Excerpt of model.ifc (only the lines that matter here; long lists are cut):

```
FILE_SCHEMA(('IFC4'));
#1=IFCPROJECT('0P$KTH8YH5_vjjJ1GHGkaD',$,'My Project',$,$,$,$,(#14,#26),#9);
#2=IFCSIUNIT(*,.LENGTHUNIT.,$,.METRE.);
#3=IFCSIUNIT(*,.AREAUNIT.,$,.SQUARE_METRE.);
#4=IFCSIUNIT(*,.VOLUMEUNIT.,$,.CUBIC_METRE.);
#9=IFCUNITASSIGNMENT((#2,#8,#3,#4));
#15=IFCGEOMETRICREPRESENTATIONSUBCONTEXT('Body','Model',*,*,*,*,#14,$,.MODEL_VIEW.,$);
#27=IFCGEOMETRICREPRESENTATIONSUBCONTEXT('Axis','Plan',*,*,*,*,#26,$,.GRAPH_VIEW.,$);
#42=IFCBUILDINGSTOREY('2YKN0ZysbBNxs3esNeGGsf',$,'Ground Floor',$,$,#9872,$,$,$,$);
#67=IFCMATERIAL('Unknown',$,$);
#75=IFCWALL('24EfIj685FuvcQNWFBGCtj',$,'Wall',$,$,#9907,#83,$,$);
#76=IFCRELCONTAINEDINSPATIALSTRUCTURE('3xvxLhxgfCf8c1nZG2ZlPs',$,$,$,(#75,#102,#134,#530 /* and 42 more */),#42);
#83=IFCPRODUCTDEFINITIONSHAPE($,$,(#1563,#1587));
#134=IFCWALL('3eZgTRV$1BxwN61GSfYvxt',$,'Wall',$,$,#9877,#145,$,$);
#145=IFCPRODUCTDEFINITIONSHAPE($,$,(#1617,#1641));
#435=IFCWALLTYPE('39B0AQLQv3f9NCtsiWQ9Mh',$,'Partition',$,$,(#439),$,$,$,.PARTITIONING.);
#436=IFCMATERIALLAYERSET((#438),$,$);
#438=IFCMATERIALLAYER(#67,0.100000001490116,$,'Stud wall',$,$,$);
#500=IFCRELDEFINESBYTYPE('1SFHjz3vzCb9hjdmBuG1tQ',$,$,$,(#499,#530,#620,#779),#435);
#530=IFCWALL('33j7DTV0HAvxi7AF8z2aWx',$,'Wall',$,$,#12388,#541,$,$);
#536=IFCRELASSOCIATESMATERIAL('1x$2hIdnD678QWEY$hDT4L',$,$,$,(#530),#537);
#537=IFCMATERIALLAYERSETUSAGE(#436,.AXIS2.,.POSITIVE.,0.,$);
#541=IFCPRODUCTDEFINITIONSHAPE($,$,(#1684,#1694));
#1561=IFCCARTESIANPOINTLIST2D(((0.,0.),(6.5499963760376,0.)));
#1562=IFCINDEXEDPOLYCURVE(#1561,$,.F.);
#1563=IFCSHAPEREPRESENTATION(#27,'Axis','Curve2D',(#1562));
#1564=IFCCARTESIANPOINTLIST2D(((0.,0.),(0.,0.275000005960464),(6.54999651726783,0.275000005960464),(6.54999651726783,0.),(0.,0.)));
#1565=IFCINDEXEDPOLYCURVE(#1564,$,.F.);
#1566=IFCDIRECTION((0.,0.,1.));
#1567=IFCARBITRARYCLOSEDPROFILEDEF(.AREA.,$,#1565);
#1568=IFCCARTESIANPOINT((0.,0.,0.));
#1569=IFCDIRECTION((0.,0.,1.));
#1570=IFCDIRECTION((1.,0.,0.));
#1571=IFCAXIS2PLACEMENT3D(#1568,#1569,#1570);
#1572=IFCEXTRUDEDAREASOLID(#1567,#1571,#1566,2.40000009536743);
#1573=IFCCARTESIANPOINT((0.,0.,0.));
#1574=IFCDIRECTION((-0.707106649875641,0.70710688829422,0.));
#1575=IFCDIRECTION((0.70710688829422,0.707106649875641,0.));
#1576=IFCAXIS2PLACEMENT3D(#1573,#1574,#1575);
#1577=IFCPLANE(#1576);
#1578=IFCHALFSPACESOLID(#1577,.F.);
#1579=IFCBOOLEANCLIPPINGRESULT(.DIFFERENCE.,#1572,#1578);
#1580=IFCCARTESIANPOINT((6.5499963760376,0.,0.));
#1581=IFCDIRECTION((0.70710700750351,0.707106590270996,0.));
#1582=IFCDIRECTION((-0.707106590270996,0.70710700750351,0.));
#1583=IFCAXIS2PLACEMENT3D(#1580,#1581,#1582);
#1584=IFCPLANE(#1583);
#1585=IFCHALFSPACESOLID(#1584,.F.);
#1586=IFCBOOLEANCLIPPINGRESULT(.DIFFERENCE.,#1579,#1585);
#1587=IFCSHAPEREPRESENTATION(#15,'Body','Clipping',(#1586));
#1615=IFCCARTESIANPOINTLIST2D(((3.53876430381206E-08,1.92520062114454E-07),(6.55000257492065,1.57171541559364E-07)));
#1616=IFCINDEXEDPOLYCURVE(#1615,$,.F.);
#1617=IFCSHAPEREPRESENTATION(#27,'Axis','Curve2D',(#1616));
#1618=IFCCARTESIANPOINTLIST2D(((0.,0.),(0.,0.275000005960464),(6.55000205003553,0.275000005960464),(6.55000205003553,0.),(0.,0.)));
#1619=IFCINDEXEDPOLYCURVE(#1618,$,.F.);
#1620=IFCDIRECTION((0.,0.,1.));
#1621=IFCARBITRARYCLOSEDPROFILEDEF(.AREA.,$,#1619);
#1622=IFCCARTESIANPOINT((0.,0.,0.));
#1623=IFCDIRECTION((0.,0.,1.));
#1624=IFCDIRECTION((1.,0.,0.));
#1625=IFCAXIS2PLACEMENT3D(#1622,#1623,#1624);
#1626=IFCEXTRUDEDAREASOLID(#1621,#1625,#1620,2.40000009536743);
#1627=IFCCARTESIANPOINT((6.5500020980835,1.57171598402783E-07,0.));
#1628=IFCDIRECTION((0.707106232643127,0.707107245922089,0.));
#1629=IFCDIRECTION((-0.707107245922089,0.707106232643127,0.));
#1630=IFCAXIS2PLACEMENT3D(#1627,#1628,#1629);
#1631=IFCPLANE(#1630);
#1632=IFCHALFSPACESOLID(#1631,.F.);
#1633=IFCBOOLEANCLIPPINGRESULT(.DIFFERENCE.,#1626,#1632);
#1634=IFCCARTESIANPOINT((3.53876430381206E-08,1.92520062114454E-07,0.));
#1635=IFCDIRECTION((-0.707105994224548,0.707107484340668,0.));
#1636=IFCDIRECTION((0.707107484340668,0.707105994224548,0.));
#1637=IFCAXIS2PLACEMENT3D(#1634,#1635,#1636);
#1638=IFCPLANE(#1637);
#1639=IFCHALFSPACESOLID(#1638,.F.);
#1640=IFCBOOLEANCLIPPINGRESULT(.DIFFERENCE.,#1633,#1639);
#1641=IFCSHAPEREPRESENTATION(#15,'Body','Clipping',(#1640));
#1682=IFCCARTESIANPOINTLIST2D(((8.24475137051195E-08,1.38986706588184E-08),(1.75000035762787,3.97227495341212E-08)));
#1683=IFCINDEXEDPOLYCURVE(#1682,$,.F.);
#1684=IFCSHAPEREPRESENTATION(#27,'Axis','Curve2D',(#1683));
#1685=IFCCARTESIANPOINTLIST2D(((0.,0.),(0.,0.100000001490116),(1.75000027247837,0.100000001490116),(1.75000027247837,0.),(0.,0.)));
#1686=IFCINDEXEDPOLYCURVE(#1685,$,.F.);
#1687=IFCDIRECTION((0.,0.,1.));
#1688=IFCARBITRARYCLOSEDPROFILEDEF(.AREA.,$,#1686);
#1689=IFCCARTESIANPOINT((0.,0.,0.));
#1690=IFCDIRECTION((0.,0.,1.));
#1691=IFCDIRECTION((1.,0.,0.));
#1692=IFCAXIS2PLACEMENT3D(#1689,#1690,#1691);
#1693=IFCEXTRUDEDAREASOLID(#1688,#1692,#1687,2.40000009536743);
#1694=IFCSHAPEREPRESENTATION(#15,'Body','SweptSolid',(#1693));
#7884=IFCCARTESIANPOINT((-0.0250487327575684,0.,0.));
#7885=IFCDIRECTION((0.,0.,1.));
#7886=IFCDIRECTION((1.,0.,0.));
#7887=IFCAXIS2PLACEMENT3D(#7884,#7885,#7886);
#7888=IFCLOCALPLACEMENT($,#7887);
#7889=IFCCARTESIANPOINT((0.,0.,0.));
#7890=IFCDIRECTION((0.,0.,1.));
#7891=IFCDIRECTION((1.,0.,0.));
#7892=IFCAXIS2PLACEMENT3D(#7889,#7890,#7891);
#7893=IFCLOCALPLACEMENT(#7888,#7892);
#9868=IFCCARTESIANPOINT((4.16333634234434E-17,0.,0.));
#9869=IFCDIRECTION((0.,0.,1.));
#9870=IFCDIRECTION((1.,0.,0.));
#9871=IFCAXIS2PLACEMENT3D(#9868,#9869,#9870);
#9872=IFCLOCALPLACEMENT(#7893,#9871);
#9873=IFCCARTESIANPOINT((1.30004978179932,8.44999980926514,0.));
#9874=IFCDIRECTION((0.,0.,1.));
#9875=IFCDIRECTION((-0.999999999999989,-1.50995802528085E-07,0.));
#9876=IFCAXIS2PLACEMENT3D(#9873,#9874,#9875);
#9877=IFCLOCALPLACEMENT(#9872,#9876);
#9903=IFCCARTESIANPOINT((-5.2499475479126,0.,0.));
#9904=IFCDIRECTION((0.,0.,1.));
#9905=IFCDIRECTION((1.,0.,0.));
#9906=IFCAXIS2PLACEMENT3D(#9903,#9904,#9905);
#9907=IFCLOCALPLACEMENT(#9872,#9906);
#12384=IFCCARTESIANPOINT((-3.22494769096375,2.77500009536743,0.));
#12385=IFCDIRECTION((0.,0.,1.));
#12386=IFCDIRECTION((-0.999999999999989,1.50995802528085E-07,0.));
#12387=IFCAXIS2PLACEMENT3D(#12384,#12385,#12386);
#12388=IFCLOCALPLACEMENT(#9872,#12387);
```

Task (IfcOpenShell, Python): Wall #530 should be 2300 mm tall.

```python
import ifcopenshell
import ifcopenshell.geom
import ifcopenshell.util.representation
import ifcopenshell.util.shape
import ifcopenshell.util.unit

model = ifcopenshell.open("model.ifc")
unit_scale = ifcopenshell.util.unit.calculate_unit_scale(model)
settings = ifcopenshell.geom.settings()


def volume(element):
    """Net volume in cubic metres, openings subtracted."""
    shape = ifcopenshell.geom.create_shape(settings, element)
    return ifcopenshell.util.shape.get_volume(shape.geometry)


wall = model.by_guid("33j7DTV0HAvxi7AF8z2aWx")
before = volume(wall)

body = ifcopenshell.util.representation.get_representation(wall, "Model", "Body")
solid = body.Items[0]
old_height = solid.Depth
solid.Depth = 2.3 / unit_scale
after = volume(wall)

print(f"height {old_height:g} -> {solid.Depth:g}, volume {before:.3f} -> {after:.3f} m3")

model.write("model_edited.ifc")
```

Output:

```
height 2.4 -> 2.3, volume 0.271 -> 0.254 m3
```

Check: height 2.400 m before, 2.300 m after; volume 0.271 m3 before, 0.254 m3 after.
